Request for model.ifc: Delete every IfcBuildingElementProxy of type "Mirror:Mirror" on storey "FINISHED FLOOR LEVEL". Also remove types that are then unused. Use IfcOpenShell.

First a look at what the model holds.

```python
import ifcopenshell
import ifcopenshell.util.element

model = ifcopenshell.open("model.ifc")
print(model.schema)
storey = next(s for s in model.by_type("IfcBuildingStorey") if s.Name == "FINISHED FLOOR LEVEL")
proxies = [e for e in ifcopenshell.util.element.get_decomposition(storey) if e.is_a("IfcBuildingElementProxy")]
seen = {}
for e in proxies:
    element_type = ifcopenshell.util.element.get_type(e)
    name = element_type.Name if element_type not in (None, e) else None
    seen[name] = seen.get(name, 0) + 1
for name, count in sorted(seen.items(), key=str):
    print(count, "x", name)
```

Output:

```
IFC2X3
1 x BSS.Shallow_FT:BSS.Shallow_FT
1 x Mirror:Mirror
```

```python
import ifcopenshell
import ifcopenshell.api.root
import ifcopenshell.util.element

model = ifcopenshell.open("model.ifc")

storey = next(s for s in model.by_type("IfcBuildingStorey") if s.Name == "FINISHED FLOOR LEVEL")
proxies = [e for e in ifcopenshell.util.element.get_decomposition(storey) if e.is_a("IfcBuildingElementProxy")]
targets = [e for e in proxies if (t := ifcopenshell.util.element.get_type(e)) not in (None, e) and t.Name == "Mirror:Mirror"]
types = {ifcopenshell.util.element.get_type(e) for e in targets} - {None, *targets}

for e in targets:
    ifcopenshell.api.root.remove_product(model, product=e)
print(len(targets), "removed")

unused = [t for t in types if not ifcopenshell.util.element.get_types(t)]
for t in unused:
    ifcopenshell.api.root.remove_product(model, product=t)
print(len(unused), "unused types removed")

model.write("model_edited.ifc")
```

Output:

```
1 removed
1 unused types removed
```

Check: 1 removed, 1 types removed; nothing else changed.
